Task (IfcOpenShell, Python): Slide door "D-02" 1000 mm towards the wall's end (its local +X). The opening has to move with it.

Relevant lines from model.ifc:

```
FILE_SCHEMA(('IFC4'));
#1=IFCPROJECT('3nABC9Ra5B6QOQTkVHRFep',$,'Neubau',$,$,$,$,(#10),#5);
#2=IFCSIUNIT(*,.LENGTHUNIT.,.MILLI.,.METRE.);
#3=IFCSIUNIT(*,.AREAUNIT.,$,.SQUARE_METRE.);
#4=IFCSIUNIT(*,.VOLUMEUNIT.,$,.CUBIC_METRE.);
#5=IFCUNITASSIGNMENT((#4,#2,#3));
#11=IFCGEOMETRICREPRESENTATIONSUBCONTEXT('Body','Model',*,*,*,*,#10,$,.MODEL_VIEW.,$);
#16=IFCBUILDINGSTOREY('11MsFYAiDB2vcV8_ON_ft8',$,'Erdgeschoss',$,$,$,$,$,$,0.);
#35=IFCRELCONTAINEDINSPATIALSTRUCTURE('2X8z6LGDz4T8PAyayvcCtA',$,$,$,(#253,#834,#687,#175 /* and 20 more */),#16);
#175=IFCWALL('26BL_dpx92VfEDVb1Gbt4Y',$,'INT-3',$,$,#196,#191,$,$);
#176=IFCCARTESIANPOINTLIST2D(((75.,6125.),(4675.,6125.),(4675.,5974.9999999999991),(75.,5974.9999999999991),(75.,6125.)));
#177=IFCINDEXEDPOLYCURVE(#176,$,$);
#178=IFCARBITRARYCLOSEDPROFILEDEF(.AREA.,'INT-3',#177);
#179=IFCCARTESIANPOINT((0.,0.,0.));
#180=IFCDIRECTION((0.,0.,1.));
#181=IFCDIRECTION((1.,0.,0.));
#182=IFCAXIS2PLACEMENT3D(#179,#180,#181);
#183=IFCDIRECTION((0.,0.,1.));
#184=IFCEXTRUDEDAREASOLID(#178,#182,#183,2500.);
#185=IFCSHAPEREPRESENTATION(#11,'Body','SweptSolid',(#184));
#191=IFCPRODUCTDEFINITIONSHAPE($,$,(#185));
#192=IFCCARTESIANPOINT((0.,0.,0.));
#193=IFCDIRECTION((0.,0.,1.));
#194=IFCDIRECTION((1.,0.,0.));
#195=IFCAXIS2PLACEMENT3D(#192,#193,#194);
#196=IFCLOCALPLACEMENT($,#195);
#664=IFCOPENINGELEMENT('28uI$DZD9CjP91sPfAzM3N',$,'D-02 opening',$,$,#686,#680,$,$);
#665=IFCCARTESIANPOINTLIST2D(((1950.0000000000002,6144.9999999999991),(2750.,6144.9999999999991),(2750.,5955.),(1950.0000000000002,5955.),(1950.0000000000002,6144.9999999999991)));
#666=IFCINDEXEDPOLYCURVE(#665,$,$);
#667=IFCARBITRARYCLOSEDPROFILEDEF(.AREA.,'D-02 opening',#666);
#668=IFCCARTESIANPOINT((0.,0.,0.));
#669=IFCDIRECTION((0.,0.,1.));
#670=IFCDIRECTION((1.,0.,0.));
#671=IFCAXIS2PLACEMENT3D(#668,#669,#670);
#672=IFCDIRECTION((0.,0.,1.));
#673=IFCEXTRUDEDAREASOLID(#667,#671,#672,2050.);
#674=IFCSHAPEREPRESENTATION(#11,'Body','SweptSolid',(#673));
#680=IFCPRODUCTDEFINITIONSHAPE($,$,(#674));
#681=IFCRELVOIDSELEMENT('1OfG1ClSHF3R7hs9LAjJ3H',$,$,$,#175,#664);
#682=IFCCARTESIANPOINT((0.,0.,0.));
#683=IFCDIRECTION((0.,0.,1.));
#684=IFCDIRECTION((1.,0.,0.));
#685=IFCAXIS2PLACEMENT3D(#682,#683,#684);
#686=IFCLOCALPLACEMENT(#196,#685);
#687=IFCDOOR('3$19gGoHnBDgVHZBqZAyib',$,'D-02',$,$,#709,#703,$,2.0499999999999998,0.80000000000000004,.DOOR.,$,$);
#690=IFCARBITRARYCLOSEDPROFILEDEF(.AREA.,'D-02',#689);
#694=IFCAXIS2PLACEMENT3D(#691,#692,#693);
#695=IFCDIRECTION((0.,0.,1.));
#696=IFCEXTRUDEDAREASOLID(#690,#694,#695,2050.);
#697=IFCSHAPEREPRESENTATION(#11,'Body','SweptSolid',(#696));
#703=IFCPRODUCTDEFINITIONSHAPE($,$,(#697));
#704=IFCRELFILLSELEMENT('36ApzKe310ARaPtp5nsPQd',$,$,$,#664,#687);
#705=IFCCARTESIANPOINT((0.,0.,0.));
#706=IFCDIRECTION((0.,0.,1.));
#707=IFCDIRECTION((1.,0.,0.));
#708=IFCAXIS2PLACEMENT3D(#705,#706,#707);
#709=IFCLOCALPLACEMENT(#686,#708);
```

```python
import ifcopenshell
import ifcopenshell.api.geometry
import ifcopenshell.util.placement

model = ifcopenshell.open("model.ifc")

door = model.by_guid("3$19gGoHnBDgVHZBqZAyib")
opening = door.FillsVoids[0].RelatingOpeningElement
wall = opening.VoidsElements[0].RelatingBuildingElement

wall_matrix = ifcopenshell.util.placement.get_local_placement(wall.ObjectPlacement)
shift = wall_matrix[:3, 0] * 1000.0
before = ifcopenshell.util.placement.get_local_placement(door.ObjectPlacement)[:3, 3].copy()

# The door is placed relative to its opening, so it follows when the opening moves.
matrix = ifcopenshell.util.placement.get_local_placement(opening.ObjectPlacement)
matrix[:3, 3] += shift
ifcopenshell.api.geometry.edit_object_placement(
    model, product=opening, matrix=matrix, is_si=False, should_transform_children=True
)

after = ifcopenshell.util.placement.get_local_placement(door.ObjectPlacement)[:3, 3]
print("door moved by", (after - before).round(3) + 0.0)

model.write("model_edited.ifc")
```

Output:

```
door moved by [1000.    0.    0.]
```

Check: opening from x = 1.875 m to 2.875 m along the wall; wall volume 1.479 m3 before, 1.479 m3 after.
